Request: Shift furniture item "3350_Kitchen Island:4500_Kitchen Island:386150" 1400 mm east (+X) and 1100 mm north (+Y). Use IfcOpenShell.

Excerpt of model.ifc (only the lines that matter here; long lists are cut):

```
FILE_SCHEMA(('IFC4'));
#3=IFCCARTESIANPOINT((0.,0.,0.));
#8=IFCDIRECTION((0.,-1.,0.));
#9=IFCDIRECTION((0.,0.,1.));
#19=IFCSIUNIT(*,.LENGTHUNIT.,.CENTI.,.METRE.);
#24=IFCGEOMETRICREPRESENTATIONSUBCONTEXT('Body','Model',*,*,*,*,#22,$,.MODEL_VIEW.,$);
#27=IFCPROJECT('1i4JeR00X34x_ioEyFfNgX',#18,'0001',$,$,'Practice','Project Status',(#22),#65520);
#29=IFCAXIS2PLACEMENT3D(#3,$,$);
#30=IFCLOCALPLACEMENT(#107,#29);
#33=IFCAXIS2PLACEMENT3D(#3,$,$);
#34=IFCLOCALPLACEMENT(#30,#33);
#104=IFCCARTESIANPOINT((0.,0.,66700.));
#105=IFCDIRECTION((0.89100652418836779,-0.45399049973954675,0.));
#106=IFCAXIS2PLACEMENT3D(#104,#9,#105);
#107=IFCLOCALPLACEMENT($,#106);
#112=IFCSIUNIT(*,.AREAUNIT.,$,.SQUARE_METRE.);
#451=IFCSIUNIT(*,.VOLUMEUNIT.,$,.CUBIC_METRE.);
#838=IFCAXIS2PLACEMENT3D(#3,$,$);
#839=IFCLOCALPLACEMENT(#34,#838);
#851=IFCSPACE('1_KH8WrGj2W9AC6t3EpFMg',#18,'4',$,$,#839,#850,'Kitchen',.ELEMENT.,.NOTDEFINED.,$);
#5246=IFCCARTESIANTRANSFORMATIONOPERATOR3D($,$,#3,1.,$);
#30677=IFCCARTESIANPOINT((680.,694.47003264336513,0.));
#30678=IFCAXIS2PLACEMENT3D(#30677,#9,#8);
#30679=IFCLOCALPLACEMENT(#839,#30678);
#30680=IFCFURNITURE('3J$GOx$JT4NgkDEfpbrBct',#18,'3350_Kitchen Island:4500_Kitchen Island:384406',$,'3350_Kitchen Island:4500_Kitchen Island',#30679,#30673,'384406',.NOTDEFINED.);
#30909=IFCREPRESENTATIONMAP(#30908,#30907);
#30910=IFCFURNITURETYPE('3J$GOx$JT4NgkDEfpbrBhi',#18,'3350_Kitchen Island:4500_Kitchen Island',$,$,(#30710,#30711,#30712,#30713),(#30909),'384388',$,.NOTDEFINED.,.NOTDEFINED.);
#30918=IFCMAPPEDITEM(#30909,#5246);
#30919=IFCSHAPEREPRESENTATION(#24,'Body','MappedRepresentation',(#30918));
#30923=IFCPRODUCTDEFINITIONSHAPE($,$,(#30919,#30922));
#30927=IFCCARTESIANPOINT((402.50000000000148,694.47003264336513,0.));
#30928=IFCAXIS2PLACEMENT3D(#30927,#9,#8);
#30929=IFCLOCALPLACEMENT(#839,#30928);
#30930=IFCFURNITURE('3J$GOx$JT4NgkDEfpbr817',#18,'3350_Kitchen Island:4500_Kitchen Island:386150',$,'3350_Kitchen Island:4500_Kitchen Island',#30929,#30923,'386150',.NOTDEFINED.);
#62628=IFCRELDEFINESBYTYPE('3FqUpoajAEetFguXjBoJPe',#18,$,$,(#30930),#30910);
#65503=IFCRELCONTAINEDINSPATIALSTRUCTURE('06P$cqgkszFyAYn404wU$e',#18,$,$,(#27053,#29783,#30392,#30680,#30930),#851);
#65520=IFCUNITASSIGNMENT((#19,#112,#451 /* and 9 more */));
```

```python
import ifcopenshell
import ifcopenshell.api.geometry
import ifcopenshell.util.placement
import ifcopenshell.util.unit

model = ifcopenshell.open("model.ifc")
unit_scale = ifcopenshell.util.unit.calculate_unit_scale(model)

item = model.by_guid("3J$GOx$JT4NgkDEfpbr817")
matrix = ifcopenshell.util.placement.get_local_placement(item.ObjectPlacement)
matrix[0, 3] += 1.4 / unit_scale
matrix[1, 3] += 1.1 / unit_scale
ifcopenshell.api.geometry.edit_object_placement(model, product=item, matrix=matrix, is_si=False)

print(ifcopenshell.util.placement.get_local_placement(item.ObjectPlacement).round(3) + 0.0)

model.write("model_edited.ifc")
```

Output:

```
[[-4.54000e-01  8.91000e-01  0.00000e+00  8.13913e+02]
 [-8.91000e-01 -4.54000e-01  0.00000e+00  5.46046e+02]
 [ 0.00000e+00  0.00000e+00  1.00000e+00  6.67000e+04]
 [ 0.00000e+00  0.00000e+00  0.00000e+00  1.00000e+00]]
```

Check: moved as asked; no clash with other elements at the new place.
